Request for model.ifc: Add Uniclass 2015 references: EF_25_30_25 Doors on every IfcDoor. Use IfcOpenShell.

First a look at what the model holds.

```python
import ifcopenshell

model = ifcopenshell.open("model.ifc")
print(model.schema)
print("classifications:", [c.Name for c in model.by_type("IfcClassification")])
for ifc_class in ("IfcDoor", "IfcRoof", "IfcStair", "IfcWall", "IfcWindow"):
    print(ifc_class, len(model.by_type(ifc_class)))
```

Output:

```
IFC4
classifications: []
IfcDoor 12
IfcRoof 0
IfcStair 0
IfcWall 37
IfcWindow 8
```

```python
import ifcopenshell
import ifcopenshell.api.classification

model = ifcopenshell.open("model.ifc")

system = ifcopenshell.api.classification.add_classification(model, classification="Uniclass 2015")

codes = {
    "IfcDoor": ("EF_25_30_25", "Doors"),
}
for ifc_class, (code, name) in codes.items():
    products = model.by_type(ifc_class)
    ifcopenshell.api.classification.add_reference(
        model, products=products, classification=system, identification=code, name=name
    )
    print(code, len(products))

model.write("model_edited.ifc")
```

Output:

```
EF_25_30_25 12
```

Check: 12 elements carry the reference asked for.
